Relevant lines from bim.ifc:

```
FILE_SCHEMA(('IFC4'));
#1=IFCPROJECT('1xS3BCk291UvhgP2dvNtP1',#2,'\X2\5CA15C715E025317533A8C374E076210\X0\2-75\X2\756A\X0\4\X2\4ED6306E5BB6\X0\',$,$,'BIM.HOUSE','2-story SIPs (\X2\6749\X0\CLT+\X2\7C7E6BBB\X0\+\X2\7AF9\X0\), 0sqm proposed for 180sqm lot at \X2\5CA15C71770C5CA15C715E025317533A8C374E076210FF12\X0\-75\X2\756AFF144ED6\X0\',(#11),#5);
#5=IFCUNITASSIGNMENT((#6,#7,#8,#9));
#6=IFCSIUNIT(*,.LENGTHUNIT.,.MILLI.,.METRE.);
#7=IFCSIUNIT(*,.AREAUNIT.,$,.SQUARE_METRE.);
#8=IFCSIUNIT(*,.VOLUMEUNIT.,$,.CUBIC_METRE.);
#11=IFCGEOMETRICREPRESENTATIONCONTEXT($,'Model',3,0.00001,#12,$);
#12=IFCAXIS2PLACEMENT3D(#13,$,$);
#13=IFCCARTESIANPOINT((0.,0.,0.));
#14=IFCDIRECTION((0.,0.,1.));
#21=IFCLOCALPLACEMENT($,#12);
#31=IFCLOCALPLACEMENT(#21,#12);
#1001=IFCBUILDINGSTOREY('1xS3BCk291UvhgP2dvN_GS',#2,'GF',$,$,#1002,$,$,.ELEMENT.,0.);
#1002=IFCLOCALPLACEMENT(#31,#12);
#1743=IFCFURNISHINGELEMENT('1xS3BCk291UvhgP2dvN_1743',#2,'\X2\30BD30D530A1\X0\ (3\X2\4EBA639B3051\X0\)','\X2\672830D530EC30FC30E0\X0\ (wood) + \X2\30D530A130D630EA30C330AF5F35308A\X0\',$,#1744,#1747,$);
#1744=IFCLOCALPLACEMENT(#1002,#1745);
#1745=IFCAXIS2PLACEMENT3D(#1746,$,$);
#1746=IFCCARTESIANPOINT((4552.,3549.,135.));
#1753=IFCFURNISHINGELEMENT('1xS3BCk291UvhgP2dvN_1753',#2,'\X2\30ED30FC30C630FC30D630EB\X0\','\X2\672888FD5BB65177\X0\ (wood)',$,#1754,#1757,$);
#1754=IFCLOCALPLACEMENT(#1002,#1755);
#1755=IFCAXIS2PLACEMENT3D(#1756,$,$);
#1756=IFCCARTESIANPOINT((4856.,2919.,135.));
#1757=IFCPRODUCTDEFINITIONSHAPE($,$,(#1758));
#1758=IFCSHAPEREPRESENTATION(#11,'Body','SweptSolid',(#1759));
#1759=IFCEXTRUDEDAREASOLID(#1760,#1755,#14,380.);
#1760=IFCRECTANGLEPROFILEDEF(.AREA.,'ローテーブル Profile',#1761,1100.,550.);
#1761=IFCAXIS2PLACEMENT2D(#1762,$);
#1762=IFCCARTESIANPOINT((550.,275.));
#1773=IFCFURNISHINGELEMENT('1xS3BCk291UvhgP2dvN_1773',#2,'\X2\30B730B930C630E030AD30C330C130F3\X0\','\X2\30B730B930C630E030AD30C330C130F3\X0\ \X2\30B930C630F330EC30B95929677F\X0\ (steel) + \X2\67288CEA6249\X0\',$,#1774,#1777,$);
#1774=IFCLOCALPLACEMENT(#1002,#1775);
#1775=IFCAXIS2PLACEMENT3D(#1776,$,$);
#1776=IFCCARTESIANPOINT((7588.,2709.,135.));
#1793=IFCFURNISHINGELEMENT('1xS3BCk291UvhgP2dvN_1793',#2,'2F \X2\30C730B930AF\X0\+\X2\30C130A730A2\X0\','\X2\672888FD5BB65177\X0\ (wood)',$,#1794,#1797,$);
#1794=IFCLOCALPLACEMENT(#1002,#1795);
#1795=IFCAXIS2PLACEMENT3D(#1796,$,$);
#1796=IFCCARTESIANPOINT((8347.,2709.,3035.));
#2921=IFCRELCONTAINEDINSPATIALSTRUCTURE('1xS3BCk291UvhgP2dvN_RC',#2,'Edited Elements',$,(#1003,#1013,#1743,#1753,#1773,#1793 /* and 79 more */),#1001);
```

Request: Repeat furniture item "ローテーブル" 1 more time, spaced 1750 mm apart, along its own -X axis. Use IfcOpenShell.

```python
import ifcopenshell
import ifcopenshell.api.geometry
import ifcopenshell.api.root
import ifcopenshell.util.element
import ifcopenshell.util.placement

model = ifcopenshell.open("bim.ifc")


def reuse_history(source, copy):
    """copy_class also copies each property set's owner history, people and application; keep the originals."""
    for rel in copy.IsDefinedBy:
        if rel.is_a("IfcRelDefinesByProperties") and (history := rel.RelatingPropertyDefinition.OwnerHistory):
            rel.RelatingPropertyDefinition.OwnerHistory = source.OwnerHistory
            ifcopenshell.util.element.remove_deep2(model, history)


source = model.by_id(1753)
base = ifcopenshell.util.placement.get_local_placement(source.ObjectPlacement)
step = -base[:3, 0] * 1750.0

for i in range(1, 2):
    copy = ifcopenshell.api.root.copy_class(model, product=source)
    copy.Representation = ifcopenshell.util.element.copy_deep(
        model, source.Representation, exclude=["IfcGeometricRepresentationContext", "IfcRepresentationMap"]
    )
    reuse_history(source, copy)
    matrix = base.copy()
    matrix[:3, 3] += i * step
    print("added at", matrix[:3, 3].round(3) + 0.0)
    ifcopenshell.api.geometry.edit_object_placement(model, product=copy, matrix=matrix, is_si=False)

model.write("bim_rev.ifc")
```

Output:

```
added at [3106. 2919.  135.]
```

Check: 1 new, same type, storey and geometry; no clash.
